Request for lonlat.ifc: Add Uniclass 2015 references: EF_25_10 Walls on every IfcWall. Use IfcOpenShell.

First a look at what the model holds.

```python
import ifcopenshell

model = ifcopenshell.open("lonlat.ifc")
print(model.schema)
print("classifications:", [c.Name for c in model.by_type("IfcClassification")])
for ifc_class in ("IfcDoor", "IfcRoof", "IfcStair", "IfcWall", "IfcWindow"):
    print(ifc_class, len(model.by_type(ifc_class)))
```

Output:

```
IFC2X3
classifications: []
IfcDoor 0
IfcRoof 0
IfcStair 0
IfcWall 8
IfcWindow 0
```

```python
import ifcopenshell
import ifcopenshell.api.classification

model = ifcopenshell.open("lonlat.ifc")

# IFC2X3 requires Source and Edition and has no link from the project to the system.
system = model.create_entity("IfcClassification", Source="NBS", Edition="2015", Name="Uniclass 2015")

codes = {
    "IfcWall": ("EF_25_10", "Walls"),
}
for ifc_class, (code, name) in codes.items():
    products = model.by_type(ifc_class)
    ifcopenshell.api.classification.add_reference(
        model, products=products, classification=system, identification=code, name=name
    )
    print(code, len(products))

model.write("lonlat-out.ifc")
```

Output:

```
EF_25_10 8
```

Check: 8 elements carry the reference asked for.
